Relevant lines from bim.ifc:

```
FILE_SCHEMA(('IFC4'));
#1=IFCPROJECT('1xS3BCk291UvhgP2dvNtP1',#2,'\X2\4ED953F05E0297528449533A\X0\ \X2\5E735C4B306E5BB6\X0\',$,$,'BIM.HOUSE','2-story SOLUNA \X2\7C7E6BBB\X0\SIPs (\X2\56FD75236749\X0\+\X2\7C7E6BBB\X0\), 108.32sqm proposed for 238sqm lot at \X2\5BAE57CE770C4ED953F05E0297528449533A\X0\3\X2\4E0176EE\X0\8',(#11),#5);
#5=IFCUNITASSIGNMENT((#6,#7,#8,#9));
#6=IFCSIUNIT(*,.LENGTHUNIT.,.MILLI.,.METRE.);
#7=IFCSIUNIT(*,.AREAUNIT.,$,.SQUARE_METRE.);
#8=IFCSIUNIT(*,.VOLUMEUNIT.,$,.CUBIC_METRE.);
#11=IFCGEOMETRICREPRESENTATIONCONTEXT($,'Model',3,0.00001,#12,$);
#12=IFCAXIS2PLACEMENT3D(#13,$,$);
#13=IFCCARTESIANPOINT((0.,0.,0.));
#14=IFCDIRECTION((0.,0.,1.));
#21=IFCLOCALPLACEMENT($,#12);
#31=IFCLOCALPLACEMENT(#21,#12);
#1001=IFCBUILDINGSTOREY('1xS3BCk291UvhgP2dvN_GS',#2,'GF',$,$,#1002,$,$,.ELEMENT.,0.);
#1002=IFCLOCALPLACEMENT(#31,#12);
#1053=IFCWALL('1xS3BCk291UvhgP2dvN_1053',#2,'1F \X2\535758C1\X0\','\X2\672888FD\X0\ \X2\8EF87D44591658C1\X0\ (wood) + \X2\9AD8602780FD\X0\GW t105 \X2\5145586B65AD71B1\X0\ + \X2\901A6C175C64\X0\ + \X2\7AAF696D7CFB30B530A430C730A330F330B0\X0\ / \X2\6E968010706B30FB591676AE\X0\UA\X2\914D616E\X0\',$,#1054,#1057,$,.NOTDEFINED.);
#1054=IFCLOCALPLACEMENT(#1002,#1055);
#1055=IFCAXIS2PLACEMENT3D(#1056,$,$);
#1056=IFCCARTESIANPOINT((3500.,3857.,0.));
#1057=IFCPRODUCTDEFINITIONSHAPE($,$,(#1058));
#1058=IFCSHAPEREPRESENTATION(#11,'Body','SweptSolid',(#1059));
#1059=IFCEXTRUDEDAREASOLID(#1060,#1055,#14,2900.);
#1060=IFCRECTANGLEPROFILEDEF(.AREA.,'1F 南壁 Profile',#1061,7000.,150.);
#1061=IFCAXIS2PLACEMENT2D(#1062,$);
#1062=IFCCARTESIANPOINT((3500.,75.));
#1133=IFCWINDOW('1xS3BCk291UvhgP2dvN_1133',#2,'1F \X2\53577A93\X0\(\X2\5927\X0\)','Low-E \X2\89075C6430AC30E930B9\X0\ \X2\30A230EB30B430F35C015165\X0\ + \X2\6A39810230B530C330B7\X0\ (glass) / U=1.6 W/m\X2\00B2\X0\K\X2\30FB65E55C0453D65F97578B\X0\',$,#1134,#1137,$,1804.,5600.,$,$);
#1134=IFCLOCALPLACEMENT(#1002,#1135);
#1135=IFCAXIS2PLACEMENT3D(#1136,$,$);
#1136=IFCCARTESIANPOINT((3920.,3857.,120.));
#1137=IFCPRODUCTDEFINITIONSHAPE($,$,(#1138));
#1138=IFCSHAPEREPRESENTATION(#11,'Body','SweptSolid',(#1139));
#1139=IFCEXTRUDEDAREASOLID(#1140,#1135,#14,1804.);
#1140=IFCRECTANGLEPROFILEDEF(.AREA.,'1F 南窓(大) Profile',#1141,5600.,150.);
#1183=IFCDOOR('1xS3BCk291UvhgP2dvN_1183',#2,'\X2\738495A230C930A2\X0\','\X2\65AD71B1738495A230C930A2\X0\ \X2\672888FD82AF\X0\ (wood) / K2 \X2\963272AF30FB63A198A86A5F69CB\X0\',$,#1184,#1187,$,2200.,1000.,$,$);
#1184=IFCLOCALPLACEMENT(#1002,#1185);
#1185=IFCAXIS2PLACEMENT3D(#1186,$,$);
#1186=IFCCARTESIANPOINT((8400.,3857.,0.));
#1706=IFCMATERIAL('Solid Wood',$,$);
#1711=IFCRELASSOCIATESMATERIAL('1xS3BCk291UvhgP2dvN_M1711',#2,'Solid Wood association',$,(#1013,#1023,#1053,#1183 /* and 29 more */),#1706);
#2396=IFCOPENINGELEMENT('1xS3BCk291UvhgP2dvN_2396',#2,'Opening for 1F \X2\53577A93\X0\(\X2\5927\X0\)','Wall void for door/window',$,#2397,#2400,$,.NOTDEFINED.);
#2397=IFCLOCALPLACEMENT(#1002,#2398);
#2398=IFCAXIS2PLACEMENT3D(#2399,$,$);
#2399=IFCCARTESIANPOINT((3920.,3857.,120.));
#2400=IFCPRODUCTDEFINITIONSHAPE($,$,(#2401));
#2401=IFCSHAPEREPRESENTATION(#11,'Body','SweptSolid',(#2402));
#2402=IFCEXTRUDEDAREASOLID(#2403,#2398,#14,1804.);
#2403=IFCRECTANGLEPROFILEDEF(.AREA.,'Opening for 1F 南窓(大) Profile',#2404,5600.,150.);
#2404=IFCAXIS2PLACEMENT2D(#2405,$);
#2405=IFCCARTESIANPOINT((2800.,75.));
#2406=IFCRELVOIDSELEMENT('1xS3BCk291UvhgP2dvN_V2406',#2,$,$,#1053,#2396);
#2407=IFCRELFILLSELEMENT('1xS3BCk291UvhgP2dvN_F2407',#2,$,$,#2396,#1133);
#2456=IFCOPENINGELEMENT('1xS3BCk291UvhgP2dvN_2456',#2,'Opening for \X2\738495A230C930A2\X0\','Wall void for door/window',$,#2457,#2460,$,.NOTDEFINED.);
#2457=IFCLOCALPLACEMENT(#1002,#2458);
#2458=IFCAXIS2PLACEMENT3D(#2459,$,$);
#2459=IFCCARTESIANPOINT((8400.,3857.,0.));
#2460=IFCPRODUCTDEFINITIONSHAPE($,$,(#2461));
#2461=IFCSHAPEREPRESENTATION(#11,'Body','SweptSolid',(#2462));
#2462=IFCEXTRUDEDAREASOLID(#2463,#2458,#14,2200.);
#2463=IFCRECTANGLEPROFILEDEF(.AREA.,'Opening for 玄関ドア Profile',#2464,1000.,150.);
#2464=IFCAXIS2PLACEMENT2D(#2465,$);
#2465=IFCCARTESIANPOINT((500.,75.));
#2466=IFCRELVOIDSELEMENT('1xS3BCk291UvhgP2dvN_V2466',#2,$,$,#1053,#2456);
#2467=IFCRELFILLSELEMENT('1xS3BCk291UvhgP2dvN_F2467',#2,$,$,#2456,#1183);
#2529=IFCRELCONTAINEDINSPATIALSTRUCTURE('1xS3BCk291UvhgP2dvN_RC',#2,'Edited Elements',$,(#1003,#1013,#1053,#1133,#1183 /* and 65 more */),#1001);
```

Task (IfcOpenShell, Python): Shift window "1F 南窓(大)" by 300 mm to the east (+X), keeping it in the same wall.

```python
import ifcopenshell
import ifcopenshell.api.geometry
import ifcopenshell.util.placement
import ifcopenshell.util.unit

model = ifcopenshell.open("bim.ifc")
unit_scale = ifcopenshell.util.unit.calculate_unit_scale(model)

window = model.by_id(1133)
opening = window.FillsVoids[0].RelatingOpeningElement
wall = opening.VoidsElements[0].RelatingBuildingElement

wall_matrix = ifcopenshell.util.placement.get_local_placement(wall.ObjectPlacement)
shift = wall_matrix[:3, 0] * 0.3 / unit_scale
before = ifcopenshell.util.placement.get_local_placement(window.ObjectPlacement)[:3, 3].copy()

# The window is not placed relative to its opening, so move both.
for product in (opening, window):
    matrix = ifcopenshell.util.placement.get_local_placement(product.ObjectPlacement)
    matrix[:3, 3] += shift
    ifcopenshell.api.geometry.edit_object_placement(model, product=product, matrix=matrix, is_si=False)

after = ifcopenshell.util.placement.get_local_placement(window.ObjectPlacement)[:3, 3]
print("window moved by", (after - before).round(3) + 0.0)

model.write("bim_rev.ifc")
```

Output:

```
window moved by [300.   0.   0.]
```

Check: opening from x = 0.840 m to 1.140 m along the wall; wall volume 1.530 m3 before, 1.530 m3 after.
